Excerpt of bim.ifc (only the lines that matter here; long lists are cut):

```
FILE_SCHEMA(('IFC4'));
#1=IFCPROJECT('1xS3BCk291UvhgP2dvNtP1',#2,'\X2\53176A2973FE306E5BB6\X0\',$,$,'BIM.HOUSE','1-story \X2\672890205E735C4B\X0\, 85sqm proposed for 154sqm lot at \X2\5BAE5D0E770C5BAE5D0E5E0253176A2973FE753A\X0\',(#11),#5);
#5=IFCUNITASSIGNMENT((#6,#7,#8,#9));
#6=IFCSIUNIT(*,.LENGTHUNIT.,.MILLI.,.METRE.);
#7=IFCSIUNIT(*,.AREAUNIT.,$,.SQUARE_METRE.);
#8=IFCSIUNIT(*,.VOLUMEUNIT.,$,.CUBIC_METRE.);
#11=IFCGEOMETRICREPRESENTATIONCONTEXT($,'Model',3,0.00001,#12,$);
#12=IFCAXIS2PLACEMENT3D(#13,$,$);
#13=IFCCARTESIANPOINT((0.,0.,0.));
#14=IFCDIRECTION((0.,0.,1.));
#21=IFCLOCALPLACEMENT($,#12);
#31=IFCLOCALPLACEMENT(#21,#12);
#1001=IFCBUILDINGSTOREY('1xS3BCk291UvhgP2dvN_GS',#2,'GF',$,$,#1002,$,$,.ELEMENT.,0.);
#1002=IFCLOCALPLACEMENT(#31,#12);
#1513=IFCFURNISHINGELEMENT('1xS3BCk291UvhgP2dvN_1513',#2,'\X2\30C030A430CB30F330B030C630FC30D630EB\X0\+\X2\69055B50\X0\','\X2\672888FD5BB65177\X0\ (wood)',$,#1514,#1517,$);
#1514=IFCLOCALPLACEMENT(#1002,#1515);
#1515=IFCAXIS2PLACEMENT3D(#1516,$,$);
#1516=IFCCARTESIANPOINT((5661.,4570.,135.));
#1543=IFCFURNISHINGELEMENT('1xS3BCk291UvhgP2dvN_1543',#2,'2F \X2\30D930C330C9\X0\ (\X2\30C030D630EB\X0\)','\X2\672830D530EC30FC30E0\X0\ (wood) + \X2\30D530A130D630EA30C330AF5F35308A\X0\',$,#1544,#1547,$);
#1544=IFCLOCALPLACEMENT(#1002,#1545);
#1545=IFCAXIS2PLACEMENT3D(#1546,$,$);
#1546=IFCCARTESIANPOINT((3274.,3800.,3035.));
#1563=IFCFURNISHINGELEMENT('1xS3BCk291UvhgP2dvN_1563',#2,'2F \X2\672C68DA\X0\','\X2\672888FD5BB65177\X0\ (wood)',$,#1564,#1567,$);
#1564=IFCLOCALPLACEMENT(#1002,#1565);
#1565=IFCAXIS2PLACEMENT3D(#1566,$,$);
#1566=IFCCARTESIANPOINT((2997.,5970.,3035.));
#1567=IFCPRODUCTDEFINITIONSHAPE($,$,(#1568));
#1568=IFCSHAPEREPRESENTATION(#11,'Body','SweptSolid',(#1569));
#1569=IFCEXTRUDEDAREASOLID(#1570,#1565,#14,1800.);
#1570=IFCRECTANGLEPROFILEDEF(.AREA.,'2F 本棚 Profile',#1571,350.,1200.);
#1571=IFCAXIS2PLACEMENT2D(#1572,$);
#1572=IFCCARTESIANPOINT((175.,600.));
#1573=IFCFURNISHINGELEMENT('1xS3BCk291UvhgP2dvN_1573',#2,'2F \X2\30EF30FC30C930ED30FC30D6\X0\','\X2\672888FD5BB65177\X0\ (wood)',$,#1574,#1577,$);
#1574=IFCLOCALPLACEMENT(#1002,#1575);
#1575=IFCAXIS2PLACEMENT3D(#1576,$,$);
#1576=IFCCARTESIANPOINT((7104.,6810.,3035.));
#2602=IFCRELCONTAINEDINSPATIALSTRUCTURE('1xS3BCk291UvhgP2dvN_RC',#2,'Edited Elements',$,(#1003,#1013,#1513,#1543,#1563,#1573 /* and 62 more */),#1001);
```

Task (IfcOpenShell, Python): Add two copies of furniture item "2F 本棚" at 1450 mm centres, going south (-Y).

```python
import numpy as np
import ifcopenshell
import ifcopenshell.api.geometry
import ifcopenshell.api.root
import ifcopenshell.util.element
import ifcopenshell.util.placement
import ifcopenshell.util.unit

model = ifcopenshell.open("bim.ifc")
unit_scale = ifcopenshell.util.unit.calculate_unit_scale(model)


def reuse_history(source, copy):
    """copy_class also copies each property set's owner history, people and application; keep the originals."""
    for rel in copy.IsDefinedBy:
        if rel.is_a("IfcRelDefinesByProperties") and (history := rel.RelatingPropertyDefinition.OwnerHistory):
            rel.RelatingPropertyDefinition.OwnerHistory = source.OwnerHistory
            ifcopenshell.util.element.remove_deep2(model, history)


source = model.by_guid("1xS3BCk291UvhgP2dvN_1563")
base = ifcopenshell.util.placement.get_local_placement(source.ObjectPlacement)
step = np.array([0.0, -1.0, 0.0]) * 1.45 / unit_scale

for i in range(1, 3):
    copy = ifcopenshell.api.root.copy_class(model, product=source)
    copy.Representation = ifcopenshell.util.element.copy_deep(
        model, source.Representation, exclude=["IfcGeometricRepresentationContext", "IfcRepresentationMap"]
    )
    reuse_history(source, copy)
    matrix = base.copy()
    matrix[:3, 3] += i * step
    print("added at", matrix[:3, 3].round(3) + 0.0)
    ifcopenshell.api.geometry.edit_object_placement(model, product=copy, matrix=matrix, is_si=False)

model.write("bim_edited.ifc")
```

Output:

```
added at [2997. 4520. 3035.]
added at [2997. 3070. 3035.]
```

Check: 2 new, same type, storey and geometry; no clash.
